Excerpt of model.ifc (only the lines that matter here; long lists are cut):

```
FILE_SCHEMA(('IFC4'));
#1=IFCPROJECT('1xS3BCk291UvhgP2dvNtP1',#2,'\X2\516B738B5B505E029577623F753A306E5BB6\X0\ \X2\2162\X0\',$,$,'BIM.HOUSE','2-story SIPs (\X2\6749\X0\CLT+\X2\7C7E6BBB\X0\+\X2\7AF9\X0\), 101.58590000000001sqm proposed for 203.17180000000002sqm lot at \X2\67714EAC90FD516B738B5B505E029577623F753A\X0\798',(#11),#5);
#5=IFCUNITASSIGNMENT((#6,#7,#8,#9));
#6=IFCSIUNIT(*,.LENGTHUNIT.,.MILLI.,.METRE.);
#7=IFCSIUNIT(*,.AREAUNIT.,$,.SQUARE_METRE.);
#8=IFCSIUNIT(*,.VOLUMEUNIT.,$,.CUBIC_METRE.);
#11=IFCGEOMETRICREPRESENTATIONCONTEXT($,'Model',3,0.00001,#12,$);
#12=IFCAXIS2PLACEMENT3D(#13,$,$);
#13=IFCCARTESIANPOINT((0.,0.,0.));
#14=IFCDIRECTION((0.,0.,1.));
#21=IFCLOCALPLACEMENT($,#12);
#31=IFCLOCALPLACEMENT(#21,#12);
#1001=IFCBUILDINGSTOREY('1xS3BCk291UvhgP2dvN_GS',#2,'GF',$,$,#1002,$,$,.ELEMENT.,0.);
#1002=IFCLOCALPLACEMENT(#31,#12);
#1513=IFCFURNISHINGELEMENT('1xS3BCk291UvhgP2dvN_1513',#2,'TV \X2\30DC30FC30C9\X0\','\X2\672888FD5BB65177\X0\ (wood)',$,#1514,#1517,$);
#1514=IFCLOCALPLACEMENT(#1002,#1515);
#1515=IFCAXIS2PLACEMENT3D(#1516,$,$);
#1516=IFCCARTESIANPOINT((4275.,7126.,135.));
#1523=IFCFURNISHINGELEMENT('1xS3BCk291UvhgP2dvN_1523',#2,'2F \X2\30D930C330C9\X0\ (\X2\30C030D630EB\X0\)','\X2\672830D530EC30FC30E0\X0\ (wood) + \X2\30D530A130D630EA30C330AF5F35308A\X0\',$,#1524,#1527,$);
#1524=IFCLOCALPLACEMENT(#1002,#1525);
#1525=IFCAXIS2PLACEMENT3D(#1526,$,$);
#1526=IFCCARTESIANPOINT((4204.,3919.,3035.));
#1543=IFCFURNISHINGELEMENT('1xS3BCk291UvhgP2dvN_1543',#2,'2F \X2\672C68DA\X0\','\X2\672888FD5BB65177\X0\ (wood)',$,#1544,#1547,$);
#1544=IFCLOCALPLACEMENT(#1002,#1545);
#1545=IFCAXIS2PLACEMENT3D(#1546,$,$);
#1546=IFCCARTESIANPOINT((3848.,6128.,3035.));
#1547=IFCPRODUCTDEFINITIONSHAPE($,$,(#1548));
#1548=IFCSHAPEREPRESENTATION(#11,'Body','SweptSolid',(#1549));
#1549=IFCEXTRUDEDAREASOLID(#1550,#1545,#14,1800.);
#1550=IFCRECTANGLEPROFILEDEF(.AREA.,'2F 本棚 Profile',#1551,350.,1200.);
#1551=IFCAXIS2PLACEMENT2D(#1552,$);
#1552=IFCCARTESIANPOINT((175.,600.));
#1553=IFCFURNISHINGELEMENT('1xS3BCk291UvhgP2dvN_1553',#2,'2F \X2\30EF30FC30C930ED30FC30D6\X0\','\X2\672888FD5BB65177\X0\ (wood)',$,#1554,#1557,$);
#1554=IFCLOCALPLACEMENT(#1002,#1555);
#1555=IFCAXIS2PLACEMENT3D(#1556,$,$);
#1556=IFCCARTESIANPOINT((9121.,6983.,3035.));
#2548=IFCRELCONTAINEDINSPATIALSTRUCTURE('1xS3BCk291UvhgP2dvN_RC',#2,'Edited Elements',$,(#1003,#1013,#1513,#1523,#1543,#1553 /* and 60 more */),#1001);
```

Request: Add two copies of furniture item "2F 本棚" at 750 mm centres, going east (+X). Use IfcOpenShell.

```python
import numpy as np
import ifcopenshell
import ifcopenshell.api.geometry
import ifcopenshell.api.root
import ifcopenshell.util.element
import ifcopenshell.util.placement
import ifcopenshell.util.unit

model = ifcopenshell.open("model.ifc")
unit_scale = ifcopenshell.util.unit.calculate_unit_scale(model)


def reuse_history(source, copy):
    """copy_class also copies each property set's owner history, people and application; keep the originals."""
    for rel in copy.IsDefinedBy:
        if rel.is_a("IfcRelDefinesByProperties") and (history := rel.RelatingPropertyDefinition.OwnerHistory):
            rel.RelatingPropertyDefinition.OwnerHistory = source.OwnerHistory
            ifcopenshell.util.element.remove_deep2(model, history)


source = model.by_id(1543)
base = ifcopenshell.util.placement.get_local_placement(source.ObjectPlacement)
step = np.array([1.0, 0.0, 0.0]) * 0.75 / unit_scale

for i in range(1, 3):
    copy = ifcopenshell.api.root.copy_class(model, product=source)
    copy.Representation = ifcopenshell.util.element.copy_deep(
        model, source.Representation, exclude=["IfcGeometricRepresentationContext", "IfcRepresentationMap"]
    )
    reuse_history(source, copy)
    matrix = base.copy()
    matrix[:3, 3] += i * step
    print("added at", matrix[:3, 3].round(3) + 0.0)
    ifcopenshell.api.geometry.edit_object_placement(model, product=copy, matrix=matrix, is_si=False)

model.write("model-out.ifc")
```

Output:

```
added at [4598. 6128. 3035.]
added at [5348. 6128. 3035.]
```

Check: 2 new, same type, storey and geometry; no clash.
